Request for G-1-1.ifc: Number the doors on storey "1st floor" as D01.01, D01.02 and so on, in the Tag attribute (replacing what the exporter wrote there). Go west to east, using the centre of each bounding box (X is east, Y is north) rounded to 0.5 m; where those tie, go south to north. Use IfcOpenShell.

First a look at what the model holds.

```python
import ifcopenshell
import ifcopenshell.util.element
import ifcopenshell.util.placement

model = ifcopenshell.open("G-1-1.ifc")
print(model.schema)
storey = next(s for s in model.by_type("IfcBuildingStorey") if s.Name == "1st floor")
doors = [e for e in ifcopenshell.util.element.get_decomposition(storey) if e.is_a("IfcDoor")]
for e in sorted(doors, key=lambda e: e.id()):
    origin = ifcopenshell.util.placement.get_local_placement(e.ObjectPlacement)[:3, 3]
    print(e.id(), e.Tag, e.Name, origin.round(2) + 0.0, sep=" | ")
```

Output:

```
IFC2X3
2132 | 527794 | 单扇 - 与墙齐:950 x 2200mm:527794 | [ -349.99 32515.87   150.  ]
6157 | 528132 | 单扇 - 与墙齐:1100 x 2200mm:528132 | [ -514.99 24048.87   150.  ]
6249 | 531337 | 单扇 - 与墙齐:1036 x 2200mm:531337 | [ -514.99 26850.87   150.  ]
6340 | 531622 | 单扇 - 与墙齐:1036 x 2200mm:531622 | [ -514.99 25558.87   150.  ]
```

```python
import ifcopenshell
import ifcopenshell.geom
import ifcopenshell.util.element
import ifcopenshell.util.shape

model = ifcopenshell.open("G-1-1.ifc")
settings = ifcopenshell.geom.settings()
settings.set("use-world-coords", True)


def centre(element):
    shape = ifcopenshell.geom.create_shape(settings, element)
    return ifcopenshell.util.shape.get_bbox_centroid(shape.geometry)


storey = next(s for s in model.by_type("IfcBuildingStorey") if s.Name == "1st floor")
doors = [e for e in ifcopenshell.util.element.get_decomposition(storey) if e.is_a("IfcDoor")]

# Insertion points can sit at a corner or the storey origin, so sort by the geometry (in metres).
centres = {e: centre(e) for e in doors}
doors.sort(key=lambda e: (round(centres[e][0] / 0.5), centres[e][1]))

for i, e in enumerate(doors, start=1):
    number = f"D01.{i:02d}"
    e.Tag = number
    print(e.id(), number)

model.write("G-1-1_rev.ifc")
```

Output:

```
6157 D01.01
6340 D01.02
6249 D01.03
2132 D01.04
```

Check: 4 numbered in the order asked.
